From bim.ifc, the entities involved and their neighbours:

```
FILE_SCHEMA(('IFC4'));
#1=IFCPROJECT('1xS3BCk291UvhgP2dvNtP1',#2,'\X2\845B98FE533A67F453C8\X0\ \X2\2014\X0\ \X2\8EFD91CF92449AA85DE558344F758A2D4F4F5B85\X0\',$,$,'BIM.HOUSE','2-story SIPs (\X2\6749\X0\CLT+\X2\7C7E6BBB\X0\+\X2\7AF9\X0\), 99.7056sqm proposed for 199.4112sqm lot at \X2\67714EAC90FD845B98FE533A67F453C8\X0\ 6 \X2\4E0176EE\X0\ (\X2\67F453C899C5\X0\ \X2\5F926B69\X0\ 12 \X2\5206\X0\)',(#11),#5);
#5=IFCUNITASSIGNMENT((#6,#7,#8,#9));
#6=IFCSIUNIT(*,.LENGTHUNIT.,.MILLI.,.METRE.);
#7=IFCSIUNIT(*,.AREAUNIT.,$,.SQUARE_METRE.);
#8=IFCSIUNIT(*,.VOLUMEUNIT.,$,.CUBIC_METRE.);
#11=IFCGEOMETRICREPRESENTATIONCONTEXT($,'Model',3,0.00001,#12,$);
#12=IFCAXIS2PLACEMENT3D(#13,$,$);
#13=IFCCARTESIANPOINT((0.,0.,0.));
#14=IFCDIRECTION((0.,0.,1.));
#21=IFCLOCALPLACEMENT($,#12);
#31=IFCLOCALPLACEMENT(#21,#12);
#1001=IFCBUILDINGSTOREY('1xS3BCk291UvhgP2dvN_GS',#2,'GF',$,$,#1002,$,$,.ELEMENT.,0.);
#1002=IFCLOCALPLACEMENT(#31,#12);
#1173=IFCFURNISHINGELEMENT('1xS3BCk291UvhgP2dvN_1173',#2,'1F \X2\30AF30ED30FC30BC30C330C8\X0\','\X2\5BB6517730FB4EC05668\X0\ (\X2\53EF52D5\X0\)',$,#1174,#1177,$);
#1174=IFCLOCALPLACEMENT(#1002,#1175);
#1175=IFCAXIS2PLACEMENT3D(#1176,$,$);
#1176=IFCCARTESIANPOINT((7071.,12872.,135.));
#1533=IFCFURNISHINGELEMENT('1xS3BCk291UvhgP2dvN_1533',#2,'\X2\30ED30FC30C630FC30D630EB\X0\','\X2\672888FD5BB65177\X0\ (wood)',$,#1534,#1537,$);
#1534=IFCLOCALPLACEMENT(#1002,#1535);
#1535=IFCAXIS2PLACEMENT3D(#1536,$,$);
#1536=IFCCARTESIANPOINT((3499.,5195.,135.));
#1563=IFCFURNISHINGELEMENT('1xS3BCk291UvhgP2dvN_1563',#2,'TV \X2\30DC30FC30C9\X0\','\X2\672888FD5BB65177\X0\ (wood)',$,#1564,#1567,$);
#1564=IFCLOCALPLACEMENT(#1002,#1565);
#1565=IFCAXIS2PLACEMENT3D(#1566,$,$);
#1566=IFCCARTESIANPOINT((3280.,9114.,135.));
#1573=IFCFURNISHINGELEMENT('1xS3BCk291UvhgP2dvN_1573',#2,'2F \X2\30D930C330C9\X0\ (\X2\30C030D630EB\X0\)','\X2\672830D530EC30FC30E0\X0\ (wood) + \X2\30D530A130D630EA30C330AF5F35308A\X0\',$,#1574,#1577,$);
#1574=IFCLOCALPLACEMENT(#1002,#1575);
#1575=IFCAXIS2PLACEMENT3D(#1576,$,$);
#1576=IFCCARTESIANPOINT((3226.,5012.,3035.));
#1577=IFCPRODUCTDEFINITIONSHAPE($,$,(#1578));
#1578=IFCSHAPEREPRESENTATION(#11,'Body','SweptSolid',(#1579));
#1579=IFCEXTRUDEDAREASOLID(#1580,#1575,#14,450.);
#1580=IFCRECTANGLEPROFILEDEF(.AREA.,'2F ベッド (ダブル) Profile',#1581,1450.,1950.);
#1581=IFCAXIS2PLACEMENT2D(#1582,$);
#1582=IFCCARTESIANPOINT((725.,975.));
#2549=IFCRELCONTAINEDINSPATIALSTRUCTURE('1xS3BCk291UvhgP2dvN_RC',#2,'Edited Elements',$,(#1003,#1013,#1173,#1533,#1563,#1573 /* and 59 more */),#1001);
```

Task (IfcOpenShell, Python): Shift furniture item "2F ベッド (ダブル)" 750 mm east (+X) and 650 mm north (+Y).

```python
import ifcopenshell
import ifcopenshell.api.geometry
import ifcopenshell.util.placement
import ifcopenshell.util.unit

model = ifcopenshell.open("bim.ifc")
unit_scale = ifcopenshell.util.unit.calculate_unit_scale(model)

item = model.by_guid("1xS3BCk291UvhgP2dvN_1573")
matrix = ifcopenshell.util.placement.get_local_placement(item.ObjectPlacement)
matrix[0, 3] += 0.75 / unit_scale
matrix[1, 3] += 0.65 / unit_scale
ifcopenshell.api.geometry.edit_object_placement(model, product=item, matrix=matrix, is_si=False)

print(ifcopenshell.util.placement.get_local_placement(item.ObjectPlacement).round(3) + 0.0)

model.write("bim-out.ifc")
```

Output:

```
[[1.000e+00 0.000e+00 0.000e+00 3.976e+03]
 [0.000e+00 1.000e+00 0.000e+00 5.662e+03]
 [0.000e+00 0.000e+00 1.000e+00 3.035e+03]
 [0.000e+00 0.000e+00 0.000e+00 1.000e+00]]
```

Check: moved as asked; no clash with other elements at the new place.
